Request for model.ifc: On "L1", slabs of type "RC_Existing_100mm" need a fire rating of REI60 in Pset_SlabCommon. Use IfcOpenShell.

First a look at what the model holds.

```python
import ifcopenshell
import ifcopenshell.util.element

model = ifcopenshell.open("model.ifc")
print(model.schema)
storey = next(s for s in model.by_type("IfcBuildingStorey") if s.Name == "L1")
slabs = [e for e in ifcopenshell.util.element.get_decomposition(storey) if e.is_a("IfcSlab")]
seen = {}
for e in slabs:
    element_type = ifcopenshell.util.element.get_type(e)
    key = (element_type.Name if element_type != e and element_type else None, ifcopenshell.util.element.get_pset(e, "Pset_SlabCommon", "FireRating"))
    seen[key] = seen.get(key, 0) + 1
for (name, value), count in sorted(seen.items(), key=str):
    print(count, "x", name, "|", value)
```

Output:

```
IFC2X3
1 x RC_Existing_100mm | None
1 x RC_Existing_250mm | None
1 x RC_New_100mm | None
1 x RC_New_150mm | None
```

```python
import ifcopenshell
import ifcopenshell.api.pset
import ifcopenshell.util.element

model = ifcopenshell.open("model.ifc")

storey = next(s for s in model.by_type("IfcBuildingStorey") if s.Name == "L1")
slabs = [e for e in ifcopenshell.util.element.get_decomposition(storey) if e.is_a("IfcSlab")]

count = 0
for e in slabs:
    element_type = ifcopenshell.util.element.get_type(e)
    if element_type in (None, e) or element_type.Name != "RC_Existing_100mm":
        continue
    # add_pset returns the element's existing set when there is one.
    pset = ifcopenshell.api.pset.add_pset(model, product=e, name="Pset_SlabCommon")
    ifcopenshell.api.pset.edit_pset(model, pset=pset, properties={"FireRating": "REI60"})
    count += 1

print(count, "slabs updated")

model.write("model_rev.ifc")
```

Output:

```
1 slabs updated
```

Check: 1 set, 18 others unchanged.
